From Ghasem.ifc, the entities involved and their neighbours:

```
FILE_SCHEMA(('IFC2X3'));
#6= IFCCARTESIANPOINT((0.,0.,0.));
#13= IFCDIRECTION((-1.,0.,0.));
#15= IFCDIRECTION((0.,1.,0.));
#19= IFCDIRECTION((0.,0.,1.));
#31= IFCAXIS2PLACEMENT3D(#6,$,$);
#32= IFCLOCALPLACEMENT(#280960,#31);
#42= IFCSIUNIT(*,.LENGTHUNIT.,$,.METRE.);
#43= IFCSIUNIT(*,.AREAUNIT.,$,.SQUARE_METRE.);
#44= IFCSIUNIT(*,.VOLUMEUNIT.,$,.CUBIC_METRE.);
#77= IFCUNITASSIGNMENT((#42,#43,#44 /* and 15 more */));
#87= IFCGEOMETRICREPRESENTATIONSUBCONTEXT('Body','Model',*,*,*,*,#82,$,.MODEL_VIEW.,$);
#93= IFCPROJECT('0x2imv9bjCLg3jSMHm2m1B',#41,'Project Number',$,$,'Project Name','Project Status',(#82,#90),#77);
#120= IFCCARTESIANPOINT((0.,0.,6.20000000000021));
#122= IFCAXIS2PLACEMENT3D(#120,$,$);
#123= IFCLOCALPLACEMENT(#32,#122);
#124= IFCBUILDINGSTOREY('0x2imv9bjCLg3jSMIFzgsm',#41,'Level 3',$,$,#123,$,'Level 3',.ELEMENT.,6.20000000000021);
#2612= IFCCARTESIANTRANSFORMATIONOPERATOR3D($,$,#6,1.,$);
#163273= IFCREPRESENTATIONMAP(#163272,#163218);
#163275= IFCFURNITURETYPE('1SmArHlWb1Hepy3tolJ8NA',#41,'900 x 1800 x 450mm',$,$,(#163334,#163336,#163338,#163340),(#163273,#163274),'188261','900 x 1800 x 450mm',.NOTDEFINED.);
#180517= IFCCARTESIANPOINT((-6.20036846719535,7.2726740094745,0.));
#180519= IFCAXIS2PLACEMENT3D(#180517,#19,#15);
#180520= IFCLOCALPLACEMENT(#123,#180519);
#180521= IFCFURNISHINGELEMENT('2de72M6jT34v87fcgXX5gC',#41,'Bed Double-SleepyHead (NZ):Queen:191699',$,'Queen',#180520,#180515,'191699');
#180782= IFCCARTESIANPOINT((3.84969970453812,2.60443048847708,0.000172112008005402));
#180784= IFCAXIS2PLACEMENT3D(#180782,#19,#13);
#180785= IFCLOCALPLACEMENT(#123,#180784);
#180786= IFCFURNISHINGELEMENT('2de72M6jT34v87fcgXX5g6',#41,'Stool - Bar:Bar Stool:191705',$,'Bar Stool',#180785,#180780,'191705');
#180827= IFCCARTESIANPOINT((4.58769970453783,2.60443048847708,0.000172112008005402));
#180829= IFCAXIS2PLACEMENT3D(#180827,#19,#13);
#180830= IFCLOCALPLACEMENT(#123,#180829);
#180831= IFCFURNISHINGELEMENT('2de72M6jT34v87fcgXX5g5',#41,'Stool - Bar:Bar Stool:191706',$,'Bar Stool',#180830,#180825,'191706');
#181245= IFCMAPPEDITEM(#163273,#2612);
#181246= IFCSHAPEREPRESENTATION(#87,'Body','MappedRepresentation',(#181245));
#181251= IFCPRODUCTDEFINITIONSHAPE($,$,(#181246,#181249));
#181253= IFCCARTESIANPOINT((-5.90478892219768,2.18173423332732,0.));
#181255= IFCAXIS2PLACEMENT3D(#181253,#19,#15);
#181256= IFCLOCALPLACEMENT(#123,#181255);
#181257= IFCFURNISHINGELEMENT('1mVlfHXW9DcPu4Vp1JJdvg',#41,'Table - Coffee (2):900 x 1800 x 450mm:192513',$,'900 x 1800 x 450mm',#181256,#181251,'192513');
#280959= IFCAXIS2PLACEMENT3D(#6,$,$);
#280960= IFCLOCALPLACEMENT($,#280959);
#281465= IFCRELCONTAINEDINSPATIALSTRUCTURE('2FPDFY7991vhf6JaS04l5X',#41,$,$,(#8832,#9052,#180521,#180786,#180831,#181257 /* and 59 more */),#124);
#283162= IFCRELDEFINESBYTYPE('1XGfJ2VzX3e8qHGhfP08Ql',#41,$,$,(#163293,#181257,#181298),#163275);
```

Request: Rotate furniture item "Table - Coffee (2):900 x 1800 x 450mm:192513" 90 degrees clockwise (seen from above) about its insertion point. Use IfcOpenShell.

```python
import ifcopenshell
import ifcopenshell.api.geometry
import ifcopenshell.util.placement

model = ifcopenshell.open("Ghasem.ifc")

item = model.by_id(181257)
matrix = ifcopenshell.util.placement.get_local_placement(item.ObjectPlacement)
matrix = matrix @ ifcopenshell.util.placement.rotation(-90, "Z")
ifcopenshell.api.geometry.edit_object_placement(model, product=item, matrix=matrix, is_si=False)

print(ifcopenshell.util.placement.get_local_placement(item.ObjectPlacement).round(3) + 0.0)

model.write("Ghasem_v2.ifc")
```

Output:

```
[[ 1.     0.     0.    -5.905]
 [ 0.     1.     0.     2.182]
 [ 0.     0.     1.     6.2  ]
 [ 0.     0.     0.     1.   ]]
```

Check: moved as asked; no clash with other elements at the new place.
